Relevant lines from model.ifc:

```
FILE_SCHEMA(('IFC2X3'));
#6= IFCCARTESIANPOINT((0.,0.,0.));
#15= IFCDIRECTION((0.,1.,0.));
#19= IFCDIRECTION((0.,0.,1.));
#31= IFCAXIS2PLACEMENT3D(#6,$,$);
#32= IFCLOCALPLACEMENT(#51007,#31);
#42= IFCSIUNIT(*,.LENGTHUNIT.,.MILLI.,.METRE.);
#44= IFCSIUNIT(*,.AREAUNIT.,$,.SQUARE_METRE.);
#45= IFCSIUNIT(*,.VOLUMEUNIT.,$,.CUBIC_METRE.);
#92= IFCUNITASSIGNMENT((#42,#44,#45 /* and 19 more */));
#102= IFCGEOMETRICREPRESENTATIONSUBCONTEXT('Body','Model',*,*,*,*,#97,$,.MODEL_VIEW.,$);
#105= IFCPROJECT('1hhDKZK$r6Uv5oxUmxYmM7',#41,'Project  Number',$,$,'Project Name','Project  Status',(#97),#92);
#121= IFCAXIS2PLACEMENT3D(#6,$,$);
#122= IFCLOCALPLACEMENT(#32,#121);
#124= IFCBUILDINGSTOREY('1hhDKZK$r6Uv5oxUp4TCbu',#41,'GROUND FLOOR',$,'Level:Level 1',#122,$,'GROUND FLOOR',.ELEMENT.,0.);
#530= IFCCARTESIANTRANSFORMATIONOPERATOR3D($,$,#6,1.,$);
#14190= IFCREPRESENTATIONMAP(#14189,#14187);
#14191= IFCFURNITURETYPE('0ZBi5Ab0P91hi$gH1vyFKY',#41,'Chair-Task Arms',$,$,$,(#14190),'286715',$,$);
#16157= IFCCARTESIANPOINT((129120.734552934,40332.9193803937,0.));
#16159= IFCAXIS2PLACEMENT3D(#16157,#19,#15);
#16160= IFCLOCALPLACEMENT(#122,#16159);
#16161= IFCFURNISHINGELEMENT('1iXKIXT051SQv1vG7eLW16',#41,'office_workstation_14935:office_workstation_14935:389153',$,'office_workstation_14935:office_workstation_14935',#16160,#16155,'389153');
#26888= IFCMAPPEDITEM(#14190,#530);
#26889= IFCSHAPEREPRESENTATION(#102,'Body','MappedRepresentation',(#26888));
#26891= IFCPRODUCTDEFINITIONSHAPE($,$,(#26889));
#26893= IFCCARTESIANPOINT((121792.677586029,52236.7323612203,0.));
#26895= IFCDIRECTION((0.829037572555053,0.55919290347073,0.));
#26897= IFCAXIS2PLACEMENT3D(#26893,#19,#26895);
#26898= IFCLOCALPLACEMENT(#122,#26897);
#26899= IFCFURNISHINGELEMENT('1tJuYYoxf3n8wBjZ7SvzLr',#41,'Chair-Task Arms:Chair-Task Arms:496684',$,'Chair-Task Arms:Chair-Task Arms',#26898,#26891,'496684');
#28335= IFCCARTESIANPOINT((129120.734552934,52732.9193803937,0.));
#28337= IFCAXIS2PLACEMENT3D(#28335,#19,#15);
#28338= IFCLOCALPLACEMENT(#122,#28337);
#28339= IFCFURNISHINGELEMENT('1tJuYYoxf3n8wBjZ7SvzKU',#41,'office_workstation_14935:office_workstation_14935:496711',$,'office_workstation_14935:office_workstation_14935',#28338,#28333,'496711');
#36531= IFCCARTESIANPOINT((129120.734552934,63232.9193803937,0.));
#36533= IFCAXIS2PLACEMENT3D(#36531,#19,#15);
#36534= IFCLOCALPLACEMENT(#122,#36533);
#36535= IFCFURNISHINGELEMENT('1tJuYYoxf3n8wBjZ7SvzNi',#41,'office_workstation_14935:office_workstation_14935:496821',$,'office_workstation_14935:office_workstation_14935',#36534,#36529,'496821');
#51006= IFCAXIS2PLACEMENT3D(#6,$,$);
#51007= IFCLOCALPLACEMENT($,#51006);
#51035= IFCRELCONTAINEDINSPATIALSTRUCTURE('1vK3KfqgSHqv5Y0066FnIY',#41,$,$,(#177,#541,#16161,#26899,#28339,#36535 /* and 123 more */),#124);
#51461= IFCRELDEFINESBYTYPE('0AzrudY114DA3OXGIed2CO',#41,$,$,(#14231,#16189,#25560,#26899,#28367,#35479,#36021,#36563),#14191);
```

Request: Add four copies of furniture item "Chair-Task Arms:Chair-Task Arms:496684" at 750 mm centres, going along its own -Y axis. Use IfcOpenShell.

```python
import ifcopenshell
import ifcopenshell.api.geometry
import ifcopenshell.api.root
import ifcopenshell.util.element
import ifcopenshell.util.placement
import ifcopenshell.util.unit

model = ifcopenshell.open("model.ifc")
unit_scale = ifcopenshell.util.unit.calculate_unit_scale(model)


def reuse_history(source, copy):
    """copy_class also copies each property set's owner history, people and application; keep the originals."""
    for rel in copy.IsDefinedBy:
        if rel.is_a("IfcRelDefinesByProperties") and (history := rel.RelatingPropertyDefinition.OwnerHistory):
            rel.RelatingPropertyDefinition.OwnerHistory = source.OwnerHistory
            ifcopenshell.util.element.remove_deep2(model, history)


source = model.by_guid("1tJuYYoxf3n8wBjZ7SvzLr")
base = ifcopenshell.util.placement.get_local_placement(source.ObjectPlacement)
step = -base[:3, 1] * 0.75 / unit_scale

for i in range(1, 5):
    copy = ifcopenshell.api.root.copy_class(model, product=source)
    copy.Representation = ifcopenshell.util.element.copy_deep(
        model, source.Representation, exclude=["IfcGeometricRepresentationContext", "IfcRepresentationMap"]
    )
    copy.Name = "Chair-Task Arms:Chair-Task Arms"
    copy.Tag = None
    reuse_history(source, copy)
    matrix = base.copy()
    matrix[:3, 3] += i * step
    print("added at", matrix[:3, 3].round(3) + 0.0)
    ifcopenshell.api.geometry.edit_object_placement(model, product=copy, matrix=matrix, is_si=False)

model.write("model_v2.ifc")
```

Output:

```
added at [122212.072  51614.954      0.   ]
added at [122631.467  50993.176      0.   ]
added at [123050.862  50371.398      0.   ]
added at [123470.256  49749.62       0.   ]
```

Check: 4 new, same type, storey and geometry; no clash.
